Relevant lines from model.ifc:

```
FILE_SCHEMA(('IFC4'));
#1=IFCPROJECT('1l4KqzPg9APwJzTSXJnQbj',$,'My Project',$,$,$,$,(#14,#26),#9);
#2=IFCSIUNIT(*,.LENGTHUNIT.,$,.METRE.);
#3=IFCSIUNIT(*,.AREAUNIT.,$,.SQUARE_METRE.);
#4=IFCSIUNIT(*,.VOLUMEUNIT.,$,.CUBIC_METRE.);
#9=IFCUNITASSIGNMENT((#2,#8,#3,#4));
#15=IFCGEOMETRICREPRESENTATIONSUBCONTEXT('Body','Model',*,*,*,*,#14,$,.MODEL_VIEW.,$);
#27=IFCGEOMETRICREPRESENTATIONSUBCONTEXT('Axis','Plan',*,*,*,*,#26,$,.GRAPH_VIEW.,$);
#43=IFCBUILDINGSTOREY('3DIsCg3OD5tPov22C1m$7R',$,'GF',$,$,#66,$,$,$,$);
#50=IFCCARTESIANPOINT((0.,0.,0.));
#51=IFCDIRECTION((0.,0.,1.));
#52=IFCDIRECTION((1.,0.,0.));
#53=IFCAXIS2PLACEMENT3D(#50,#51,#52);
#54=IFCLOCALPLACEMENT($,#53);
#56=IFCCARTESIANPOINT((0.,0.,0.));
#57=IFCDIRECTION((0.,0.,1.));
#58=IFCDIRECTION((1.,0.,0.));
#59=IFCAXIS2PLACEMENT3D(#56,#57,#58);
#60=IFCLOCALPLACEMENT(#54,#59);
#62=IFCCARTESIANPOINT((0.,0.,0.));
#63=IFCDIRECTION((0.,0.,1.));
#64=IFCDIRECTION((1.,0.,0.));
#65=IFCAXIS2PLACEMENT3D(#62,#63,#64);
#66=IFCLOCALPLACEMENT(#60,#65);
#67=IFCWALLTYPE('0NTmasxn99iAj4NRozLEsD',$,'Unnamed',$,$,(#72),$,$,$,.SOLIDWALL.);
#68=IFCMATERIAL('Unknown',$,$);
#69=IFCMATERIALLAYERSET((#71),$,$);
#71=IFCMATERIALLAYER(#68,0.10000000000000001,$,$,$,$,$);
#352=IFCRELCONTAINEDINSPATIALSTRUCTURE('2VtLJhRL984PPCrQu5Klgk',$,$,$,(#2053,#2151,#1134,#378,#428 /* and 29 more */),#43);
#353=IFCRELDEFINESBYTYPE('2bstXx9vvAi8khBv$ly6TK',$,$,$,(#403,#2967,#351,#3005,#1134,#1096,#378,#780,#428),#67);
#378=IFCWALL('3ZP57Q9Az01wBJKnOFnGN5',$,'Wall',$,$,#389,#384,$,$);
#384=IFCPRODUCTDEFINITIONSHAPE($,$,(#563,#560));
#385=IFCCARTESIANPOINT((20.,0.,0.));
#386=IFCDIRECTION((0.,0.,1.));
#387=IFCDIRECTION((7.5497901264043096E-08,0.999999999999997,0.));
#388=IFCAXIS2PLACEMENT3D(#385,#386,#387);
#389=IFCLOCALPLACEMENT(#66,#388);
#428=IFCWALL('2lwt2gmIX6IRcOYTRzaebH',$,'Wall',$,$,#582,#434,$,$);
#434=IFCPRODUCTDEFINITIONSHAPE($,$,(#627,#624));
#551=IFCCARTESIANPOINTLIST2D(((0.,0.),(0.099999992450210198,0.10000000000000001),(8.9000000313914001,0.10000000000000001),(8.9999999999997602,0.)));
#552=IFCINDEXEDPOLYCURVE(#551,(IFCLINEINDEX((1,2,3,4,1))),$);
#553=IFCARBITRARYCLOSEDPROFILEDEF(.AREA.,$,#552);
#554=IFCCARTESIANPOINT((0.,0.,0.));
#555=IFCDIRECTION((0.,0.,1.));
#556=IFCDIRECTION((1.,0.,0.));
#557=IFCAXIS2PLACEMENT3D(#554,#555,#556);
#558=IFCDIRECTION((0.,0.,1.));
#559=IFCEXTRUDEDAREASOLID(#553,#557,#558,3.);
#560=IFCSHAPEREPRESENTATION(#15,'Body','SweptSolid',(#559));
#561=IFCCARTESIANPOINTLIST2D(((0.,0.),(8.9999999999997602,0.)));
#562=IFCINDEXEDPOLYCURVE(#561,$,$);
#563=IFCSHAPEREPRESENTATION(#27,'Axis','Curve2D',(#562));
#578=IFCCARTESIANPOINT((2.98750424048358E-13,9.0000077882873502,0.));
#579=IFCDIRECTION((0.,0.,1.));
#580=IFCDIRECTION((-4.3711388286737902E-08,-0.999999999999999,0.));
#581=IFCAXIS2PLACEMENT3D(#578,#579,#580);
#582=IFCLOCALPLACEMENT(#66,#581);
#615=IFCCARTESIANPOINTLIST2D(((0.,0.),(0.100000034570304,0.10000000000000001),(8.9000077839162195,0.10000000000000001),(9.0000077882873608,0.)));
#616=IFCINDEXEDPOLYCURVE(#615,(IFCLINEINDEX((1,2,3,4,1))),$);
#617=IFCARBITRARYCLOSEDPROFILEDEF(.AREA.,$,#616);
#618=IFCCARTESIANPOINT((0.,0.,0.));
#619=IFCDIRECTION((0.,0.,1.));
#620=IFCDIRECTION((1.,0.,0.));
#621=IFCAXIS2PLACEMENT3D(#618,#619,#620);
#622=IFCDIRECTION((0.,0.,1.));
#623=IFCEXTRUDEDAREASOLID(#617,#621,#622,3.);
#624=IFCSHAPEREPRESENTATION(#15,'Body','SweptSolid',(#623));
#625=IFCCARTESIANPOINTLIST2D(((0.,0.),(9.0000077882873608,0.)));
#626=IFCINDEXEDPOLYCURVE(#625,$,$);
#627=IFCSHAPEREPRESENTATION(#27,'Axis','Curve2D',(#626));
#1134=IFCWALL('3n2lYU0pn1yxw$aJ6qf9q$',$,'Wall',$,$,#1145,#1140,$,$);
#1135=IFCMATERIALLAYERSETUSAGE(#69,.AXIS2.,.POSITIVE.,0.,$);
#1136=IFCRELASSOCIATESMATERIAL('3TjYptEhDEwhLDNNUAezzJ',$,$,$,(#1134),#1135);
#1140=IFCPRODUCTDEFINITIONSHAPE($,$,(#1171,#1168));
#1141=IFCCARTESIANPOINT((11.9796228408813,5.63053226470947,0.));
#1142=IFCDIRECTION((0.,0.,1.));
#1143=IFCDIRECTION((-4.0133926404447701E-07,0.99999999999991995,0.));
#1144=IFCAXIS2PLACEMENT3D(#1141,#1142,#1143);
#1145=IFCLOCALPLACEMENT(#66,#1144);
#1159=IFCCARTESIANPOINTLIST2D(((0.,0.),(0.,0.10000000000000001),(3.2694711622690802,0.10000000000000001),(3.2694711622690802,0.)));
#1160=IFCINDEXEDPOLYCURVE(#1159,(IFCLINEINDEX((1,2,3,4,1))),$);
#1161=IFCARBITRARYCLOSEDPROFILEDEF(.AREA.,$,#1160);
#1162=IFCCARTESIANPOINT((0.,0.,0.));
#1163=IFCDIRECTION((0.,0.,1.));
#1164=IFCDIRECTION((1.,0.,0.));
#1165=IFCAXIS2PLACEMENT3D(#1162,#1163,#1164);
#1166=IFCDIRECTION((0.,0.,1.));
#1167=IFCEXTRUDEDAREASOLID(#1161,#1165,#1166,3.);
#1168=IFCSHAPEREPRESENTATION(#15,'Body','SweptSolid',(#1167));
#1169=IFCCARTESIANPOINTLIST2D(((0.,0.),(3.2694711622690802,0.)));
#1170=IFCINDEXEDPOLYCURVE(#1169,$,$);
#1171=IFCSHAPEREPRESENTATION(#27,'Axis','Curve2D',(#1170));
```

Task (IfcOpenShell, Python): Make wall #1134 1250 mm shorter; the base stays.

```python
import ifcopenshell
import ifcopenshell.geom
import ifcopenshell.util.representation
import ifcopenshell.util.shape
import ifcopenshell.util.unit

model = ifcopenshell.open("model.ifc")
unit_scale = ifcopenshell.util.unit.calculate_unit_scale(model)
settings = ifcopenshell.geom.settings()


def volume(element):
    """Net volume in cubic metres, openings subtracted."""
    shape = ifcopenshell.geom.create_shape(settings, element)
    return ifcopenshell.util.shape.get_volume(shape.geometry)


wall = model.by_guid("3n2lYU0pn1yxw$aJ6qf9q$")
before = volume(wall)

body = ifcopenshell.util.representation.get_representation(wall, "Model", "Body")
solid = body.Items[0]
old_height = solid.Depth
solid.Depth -= 1.25 / unit_scale
after = volume(wall)

print(f"height {old_height:g} -> {solid.Depth:g}, volume {before:.3f} -> {after:.3f} m3")

model.write("model_rev.ifc")
```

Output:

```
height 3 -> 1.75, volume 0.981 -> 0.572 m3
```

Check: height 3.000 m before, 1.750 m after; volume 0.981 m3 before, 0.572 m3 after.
